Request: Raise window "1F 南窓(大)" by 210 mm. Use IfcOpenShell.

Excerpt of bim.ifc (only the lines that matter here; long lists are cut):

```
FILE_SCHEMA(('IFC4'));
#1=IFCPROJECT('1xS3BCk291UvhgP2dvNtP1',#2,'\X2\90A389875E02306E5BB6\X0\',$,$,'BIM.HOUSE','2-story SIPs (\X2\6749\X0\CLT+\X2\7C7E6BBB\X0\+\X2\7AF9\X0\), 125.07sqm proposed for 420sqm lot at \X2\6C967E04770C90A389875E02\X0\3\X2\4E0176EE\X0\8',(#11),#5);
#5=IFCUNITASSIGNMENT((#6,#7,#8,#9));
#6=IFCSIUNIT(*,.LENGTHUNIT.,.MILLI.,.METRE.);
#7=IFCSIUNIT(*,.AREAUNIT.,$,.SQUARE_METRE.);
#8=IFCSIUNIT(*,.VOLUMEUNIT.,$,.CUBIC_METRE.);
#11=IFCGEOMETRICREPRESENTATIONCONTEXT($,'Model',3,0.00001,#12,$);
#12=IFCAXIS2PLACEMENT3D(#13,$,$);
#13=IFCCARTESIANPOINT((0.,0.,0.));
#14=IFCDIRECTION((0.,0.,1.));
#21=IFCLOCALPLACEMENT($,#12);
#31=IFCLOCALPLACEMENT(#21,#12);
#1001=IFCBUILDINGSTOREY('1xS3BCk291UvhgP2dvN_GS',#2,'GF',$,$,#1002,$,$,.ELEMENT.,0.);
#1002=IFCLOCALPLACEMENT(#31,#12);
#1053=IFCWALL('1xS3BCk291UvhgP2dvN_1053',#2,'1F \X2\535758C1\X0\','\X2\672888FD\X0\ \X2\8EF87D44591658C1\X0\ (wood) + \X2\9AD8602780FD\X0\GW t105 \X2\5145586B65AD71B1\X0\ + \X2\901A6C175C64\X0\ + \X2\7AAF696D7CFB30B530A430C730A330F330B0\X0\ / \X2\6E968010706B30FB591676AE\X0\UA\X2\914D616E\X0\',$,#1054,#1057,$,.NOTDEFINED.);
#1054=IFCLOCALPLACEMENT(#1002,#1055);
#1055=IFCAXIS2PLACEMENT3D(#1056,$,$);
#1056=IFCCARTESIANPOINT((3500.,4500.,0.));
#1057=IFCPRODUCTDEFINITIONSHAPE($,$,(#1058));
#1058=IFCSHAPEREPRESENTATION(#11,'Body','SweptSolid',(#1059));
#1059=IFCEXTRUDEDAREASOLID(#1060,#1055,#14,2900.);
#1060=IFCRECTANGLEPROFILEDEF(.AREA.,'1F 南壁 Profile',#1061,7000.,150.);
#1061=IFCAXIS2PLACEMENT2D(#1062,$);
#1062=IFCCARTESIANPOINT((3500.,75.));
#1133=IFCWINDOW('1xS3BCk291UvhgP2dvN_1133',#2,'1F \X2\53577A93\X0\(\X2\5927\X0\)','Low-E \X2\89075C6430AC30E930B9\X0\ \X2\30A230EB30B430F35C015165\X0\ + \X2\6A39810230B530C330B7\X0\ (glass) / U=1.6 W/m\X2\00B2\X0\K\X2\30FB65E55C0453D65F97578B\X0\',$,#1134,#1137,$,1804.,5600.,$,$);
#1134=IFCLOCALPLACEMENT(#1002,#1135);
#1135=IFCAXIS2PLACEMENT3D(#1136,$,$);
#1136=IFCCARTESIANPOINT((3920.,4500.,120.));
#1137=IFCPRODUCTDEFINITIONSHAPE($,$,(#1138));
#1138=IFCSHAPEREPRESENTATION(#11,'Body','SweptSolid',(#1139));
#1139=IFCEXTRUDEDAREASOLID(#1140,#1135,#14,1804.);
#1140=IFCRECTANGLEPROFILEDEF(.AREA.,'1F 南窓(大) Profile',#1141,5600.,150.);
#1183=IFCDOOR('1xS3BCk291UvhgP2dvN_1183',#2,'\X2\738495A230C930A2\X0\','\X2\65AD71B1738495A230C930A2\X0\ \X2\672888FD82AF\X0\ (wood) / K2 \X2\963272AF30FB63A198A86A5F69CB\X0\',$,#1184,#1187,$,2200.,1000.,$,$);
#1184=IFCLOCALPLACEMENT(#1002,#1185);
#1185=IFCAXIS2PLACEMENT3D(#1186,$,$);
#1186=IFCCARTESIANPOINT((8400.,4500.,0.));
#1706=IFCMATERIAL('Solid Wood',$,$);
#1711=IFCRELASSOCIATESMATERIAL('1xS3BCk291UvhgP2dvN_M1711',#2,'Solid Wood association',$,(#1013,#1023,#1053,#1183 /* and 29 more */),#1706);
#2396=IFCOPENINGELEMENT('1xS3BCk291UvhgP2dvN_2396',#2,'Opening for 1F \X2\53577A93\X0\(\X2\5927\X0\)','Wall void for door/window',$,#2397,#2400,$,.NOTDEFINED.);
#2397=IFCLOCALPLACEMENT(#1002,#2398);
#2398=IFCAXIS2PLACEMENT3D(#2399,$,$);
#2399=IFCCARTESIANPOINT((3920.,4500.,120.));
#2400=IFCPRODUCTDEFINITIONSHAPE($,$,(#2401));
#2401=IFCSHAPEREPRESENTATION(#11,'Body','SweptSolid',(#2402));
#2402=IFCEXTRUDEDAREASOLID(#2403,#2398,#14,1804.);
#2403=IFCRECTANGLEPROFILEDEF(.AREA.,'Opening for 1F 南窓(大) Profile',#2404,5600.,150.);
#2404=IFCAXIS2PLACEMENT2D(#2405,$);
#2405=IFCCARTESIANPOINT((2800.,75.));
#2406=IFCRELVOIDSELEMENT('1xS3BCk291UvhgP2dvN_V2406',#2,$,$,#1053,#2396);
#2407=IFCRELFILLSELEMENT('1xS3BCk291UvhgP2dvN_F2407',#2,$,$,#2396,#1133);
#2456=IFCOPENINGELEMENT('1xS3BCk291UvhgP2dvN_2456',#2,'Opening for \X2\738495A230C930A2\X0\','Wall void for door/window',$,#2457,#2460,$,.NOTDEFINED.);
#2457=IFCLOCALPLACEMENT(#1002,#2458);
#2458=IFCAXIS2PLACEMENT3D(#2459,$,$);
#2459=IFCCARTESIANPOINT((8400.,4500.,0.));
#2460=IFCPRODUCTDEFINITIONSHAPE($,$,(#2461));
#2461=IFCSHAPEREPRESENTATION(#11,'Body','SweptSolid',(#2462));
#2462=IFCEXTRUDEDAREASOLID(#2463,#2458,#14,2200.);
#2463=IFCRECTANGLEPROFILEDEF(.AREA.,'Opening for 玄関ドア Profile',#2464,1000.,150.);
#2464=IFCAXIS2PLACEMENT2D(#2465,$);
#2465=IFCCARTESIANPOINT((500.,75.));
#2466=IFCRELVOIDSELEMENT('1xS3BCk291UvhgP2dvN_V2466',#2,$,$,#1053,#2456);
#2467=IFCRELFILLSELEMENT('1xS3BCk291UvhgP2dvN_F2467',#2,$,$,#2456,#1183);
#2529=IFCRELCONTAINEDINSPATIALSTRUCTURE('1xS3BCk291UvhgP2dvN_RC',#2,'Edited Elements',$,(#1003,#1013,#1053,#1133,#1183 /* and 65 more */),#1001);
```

```python
import numpy as np
import ifcopenshell
import ifcopenshell.api.geometry
import ifcopenshell.util.placement
import ifcopenshell.util.unit

model = ifcopenshell.open("bim.ifc")
unit_scale = ifcopenshell.util.unit.calculate_unit_scale(model)

window = model.by_id(1133)
opening = window.FillsVoids[0].RelatingOpeningElement
dz = 210.0

shift = np.array([0.0, 0.0, dz])
# The window is not placed relative to its opening, so move both.
for product in (opening, window):
    matrix = ifcopenshell.util.placement.get_local_placement(product.ObjectPlacement)
    matrix[:3, 3] += shift
    ifcopenshell.api.geometry.edit_object_placement(model, product=product, matrix=matrix, is_si=False)

print(f"moved by {dz * unit_scale:+.3f} m")

model.write("bim_rev.ifc")
```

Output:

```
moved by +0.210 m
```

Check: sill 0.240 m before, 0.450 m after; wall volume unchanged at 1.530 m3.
